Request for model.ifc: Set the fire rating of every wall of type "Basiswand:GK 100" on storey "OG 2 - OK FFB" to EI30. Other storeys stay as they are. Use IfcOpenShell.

First a look at what the model holds.

```python
import ifcopenshell
import ifcopenshell.util.element

model = ifcopenshell.open("model.ifc")
print(model.schema)
storey = next(s for s in model.by_type("IfcBuildingStorey") if s.Name == "OG 2 - OK FFB")
walls = [e for e in ifcopenshell.util.element.get_decomposition(storey) if e.is_a("IfcWall")]
seen = {}
for e in walls:
    element_type = ifcopenshell.util.element.get_type(e)
    key = (element_type.Name if element_type != e and element_type else None, ifcopenshell.util.element.get_pset(e, "Pset_WallCommon", "FireRating"))
    seen[key] = seen.get(key, 0) + 1
for (name, value), count in sorted(seen.items(), key=str):
    print(count, "x", name, "|", value)
```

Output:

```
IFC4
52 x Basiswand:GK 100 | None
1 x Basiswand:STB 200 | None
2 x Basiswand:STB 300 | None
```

```python
import ifcopenshell
import ifcopenshell.api.pset
import ifcopenshell.util.element

model = ifcopenshell.open("model.ifc")

storey = next(s for s in model.by_type("IfcBuildingStorey") if s.Name == "OG 2 - OK FFB")
walls = [e for e in ifcopenshell.util.element.get_decomposition(storey) if e.is_a("IfcWall")]

count = 0
for e in walls:
    element_type = ifcopenshell.util.element.get_type(e)
    if element_type in (None, e) or element_type.Name != "Basiswand:GK 100":
        continue
    # add_pset returns the element's existing set when there is one.
    pset = ifcopenshell.api.pset.add_pset(model, product=e, name="Pset_WallCommon")
    ifcopenshell.api.pset.edit_pset(model, pset=pset, properties={"FireRating": "EI30"})
    count += 1

print(count, "walls updated")

model.write("model_edited.ifc")
```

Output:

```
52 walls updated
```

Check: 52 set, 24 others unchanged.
